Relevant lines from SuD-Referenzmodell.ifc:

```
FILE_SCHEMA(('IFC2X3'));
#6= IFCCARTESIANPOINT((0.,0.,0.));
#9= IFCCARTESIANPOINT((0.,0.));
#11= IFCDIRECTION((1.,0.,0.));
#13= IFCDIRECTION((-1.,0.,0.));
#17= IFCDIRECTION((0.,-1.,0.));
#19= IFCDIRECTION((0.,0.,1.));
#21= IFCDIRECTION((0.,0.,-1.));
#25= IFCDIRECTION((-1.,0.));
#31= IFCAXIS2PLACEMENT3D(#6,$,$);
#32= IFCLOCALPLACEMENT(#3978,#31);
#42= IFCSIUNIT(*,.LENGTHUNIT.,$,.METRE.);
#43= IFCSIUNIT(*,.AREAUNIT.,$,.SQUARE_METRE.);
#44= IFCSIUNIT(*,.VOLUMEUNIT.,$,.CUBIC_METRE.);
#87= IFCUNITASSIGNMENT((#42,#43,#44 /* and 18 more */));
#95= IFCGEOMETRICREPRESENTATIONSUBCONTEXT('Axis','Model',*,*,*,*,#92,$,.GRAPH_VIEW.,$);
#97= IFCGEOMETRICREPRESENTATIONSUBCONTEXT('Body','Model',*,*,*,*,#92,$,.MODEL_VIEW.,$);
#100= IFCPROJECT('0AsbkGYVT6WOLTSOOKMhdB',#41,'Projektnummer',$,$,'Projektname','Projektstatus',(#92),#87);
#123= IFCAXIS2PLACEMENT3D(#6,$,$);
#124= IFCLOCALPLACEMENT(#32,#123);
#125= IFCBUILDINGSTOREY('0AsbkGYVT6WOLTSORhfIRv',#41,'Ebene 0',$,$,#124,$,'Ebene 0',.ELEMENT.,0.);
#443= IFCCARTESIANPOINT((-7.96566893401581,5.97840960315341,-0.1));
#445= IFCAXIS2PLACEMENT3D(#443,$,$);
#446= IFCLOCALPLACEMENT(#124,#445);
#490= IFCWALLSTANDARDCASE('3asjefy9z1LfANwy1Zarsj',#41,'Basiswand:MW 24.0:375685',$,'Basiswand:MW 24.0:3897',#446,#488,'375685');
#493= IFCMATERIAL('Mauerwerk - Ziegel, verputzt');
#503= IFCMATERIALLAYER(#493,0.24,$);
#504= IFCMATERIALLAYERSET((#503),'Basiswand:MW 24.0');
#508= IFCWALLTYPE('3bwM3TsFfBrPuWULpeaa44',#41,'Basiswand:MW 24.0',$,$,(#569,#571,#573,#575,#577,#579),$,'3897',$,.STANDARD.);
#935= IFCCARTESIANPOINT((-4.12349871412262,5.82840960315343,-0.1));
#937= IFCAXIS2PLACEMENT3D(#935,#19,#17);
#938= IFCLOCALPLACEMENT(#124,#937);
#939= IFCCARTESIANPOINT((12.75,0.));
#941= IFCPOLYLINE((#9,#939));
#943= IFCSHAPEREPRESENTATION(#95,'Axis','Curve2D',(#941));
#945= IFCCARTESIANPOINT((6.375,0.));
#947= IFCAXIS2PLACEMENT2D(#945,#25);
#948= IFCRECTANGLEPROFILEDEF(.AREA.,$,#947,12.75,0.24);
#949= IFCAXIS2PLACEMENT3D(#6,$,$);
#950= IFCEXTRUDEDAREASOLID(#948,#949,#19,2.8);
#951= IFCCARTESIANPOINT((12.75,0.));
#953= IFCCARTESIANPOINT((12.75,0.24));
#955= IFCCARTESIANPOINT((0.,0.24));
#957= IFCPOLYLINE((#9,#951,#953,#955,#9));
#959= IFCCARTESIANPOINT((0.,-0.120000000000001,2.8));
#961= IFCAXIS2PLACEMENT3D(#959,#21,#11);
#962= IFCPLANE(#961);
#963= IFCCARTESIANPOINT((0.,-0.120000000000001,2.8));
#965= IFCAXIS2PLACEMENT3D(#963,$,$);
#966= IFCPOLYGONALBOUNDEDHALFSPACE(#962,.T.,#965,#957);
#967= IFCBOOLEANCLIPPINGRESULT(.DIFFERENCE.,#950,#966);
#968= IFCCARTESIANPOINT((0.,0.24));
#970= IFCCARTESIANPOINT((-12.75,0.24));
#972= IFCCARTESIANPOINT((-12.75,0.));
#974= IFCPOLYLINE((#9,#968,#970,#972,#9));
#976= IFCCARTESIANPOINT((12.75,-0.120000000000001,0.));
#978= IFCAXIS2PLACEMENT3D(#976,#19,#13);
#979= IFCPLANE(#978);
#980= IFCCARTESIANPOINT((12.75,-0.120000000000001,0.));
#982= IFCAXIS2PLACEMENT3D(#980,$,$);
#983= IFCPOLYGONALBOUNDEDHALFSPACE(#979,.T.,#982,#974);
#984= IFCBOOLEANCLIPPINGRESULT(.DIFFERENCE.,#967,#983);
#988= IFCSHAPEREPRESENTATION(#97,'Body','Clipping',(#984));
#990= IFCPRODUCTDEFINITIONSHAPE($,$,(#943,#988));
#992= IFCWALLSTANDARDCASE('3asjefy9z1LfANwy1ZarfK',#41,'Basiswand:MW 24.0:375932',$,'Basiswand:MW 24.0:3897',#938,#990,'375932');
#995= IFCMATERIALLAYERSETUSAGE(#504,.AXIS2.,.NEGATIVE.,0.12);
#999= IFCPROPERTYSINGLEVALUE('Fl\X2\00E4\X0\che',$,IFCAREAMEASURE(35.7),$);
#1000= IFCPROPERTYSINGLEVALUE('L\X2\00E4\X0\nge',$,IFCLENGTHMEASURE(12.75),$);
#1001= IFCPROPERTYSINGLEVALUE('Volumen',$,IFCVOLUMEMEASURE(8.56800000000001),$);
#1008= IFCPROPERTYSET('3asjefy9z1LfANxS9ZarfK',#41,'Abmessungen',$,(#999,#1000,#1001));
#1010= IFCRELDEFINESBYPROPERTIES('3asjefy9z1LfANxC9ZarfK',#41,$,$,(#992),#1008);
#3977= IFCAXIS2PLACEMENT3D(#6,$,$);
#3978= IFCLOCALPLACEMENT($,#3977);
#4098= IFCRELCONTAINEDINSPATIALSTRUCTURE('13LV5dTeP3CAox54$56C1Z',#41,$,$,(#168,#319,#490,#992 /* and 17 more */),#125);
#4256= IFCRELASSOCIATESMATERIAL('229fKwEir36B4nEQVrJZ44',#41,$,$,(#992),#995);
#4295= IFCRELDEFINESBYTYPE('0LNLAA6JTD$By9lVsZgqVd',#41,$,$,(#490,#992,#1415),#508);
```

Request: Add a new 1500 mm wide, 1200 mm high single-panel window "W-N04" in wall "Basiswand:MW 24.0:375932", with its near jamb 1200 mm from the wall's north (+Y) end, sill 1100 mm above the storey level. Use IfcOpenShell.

```python
import numpy as np
import ifcopenshell
import ifcopenshell.api.feature
import ifcopenshell.api.geometry
import ifcopenshell.api.pset
import ifcopenshell.api.root
import ifcopenshell.api.spatial
import ifcopenshell.api.type
import ifcopenshell.geom
import ifcopenshell.util.element
import ifcopenshell.util.placement
import ifcopenshell.util.representation
import ifcopenshell.util.shape
import ifcopenshell.util.unit

model = ifcopenshell.open("SuD-Referenzmodell.ifc")
unit_scale = ifcopenshell.util.unit.calculate_unit_scale(model)
area_scale = ifcopenshell.util.unit.calculate_unit_scale(model, "AREAUNIT")
volume_scale = ifcopenshell.util.unit.calculate_unit_scale(model, "VOLUMEUNIT")
settings = ifcopenshell.geom.settings()


def volume(element):
    """Net volume in cubic metres, openings subtracted."""
    shape = ifcopenshell.geom.create_shape(settings, element)
    return ifcopenshell.util.shape.get_volume(shape.geometry)


wall = model.by_guid("3asjefy9z1LfANwy1ZarfK")
storey = ifcopenshell.util.element.get_container(wall, ifc_class="IfcBuildingStorey")
context = ifcopenshell.util.representation.get_context(model, "Model", "Body", "MODEL_VIEW")
before = volume(wall)

width, height, from_end, sill = 1.5, 1.2, 1.2, 1.1  # metres

# The wall runs along its own X axis, and the end named is its -X end.
wall_shape = ifcopenshell.geom.create_shape(settings, wall)
x, y, z = ifcopenshell.util.shape.get_vertices(wall_shape.geometry).T
start = x.min() + from_end
face, thickness = float(y.min()), float(y.max() - y.min())
wall_matrix = ifcopenshell.util.placement.get_local_placement(wall.ObjectPlacement)
level = ifcopenshell.util.placement.get_local_placement(storey.ObjectPlacement)[2, 3]


def in_wall(x, y):
    """Placement at x, y metres in the wall's axes, at sill height."""
    matrix = wall_matrix.copy()
    matrix[:, 3] = wall_matrix @ np.array([x / unit_scale, y / unit_scale, 0.0, 1.0])
    matrix[2, 3] = level + sill / unit_scale
    return matrix


# Opening: a box that overshoots both wall faces by 50 mm.
opening = ifcopenshell.api.root.create_entity(model, ifc_class="IfcOpeningElement")
box = ifcopenshell.api.geometry.add_wall_representation(
    model, context=context, length=width, height=height, thickness=thickness + 0.1
)
ifcopenshell.api.geometry.assign_representation(model, product=opening, representation=box)
ifcopenshell.api.geometry.edit_object_placement(model, product=opening, matrix=in_wall(start, face - 0.05), is_si=False)
ifcopenshell.api.feature.add_feature(model, feature=opening, element=wall)

window = ifcopenshell.api.root.create_entity(model, ifc_class="IfcWindow", name="W-N04")
window.OverallWidth, window.OverallHeight = width / unit_scale, height / unit_scale
body = ifcopenshell.api.geometry.add_window_representation(
    model,
    context=context,
    overall_width=window.OverallWidth,
    overall_height=window.OverallHeight,
    partition_type="SINGLE_PANEL",
)
ifcopenshell.api.geometry.assign_representation(model, product=window, representation=body)
ifcopenshell.api.spatial.assign_container(model, products=[window], relating_structure=storey)
fills = ifcopenshell.api.feature.add_filling(model, opening=opening, element=window)
fills.OwnerHistory = window.OwnerHistory  # required in IFC2X3

# IFC2X3 keeps the operation on the window style.
style = ifcopenshell.api.root.create_entity(model, ifc_class="IfcWindowStyle", name="W-N04")
style.OperationType, style.ConstructionType = "SINGLE_PANEL", "NOTDEFINED"
style.ParameterTakesPrecedence = style.Sizeable = False
ifcopenshell.api.type.assign_type(model, related_objects=[window], relating_type=style)

# Centre the window in the wall's thickness.
ifcopenshell.api.geometry.edit_object_placement(model, product=window, matrix=in_wall(start, face), is_si=False)
window_shape = ifcopenshell.geom.create_shape(settings, window)
depth = ifcopenshell.util.shape.get_vertices(window_shape.geometry)[:, 1]
offset = face + thickness / 2 - (depth.min() + depth.max()) / 2
ifcopenshell.api.geometry.edit_object_placement(model, product=window, matrix=in_wall(start, offset), is_si=False)

after = volume(wall)

# Update the wall's stored quantities.
pset = model.by_id(ifcopenshell.util.element.get_pset(wall, "Abmessungen", should_inherit=False)["id"])
ifcopenshell.api.pset.edit_pset(model, pset=pset, properties={
    "Fläche": model.create_entity("IfcAreaMeasure", after / thickness / area_scale),
    "Volumen": model.create_entity("IfcVolumeMeasure", after / volume_scale),
})

print(f"wall volume {before:.3f} -> {after:.3f} m3")

model.write("SuD-Referenzmodell_edited.ifc")
```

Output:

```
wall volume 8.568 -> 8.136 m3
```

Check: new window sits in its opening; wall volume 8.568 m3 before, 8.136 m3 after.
